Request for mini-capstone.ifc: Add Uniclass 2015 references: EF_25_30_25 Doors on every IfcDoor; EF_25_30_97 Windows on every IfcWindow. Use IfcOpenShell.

First a look at what the model holds.

```python
import ifcopenshell

model = ifcopenshell.open("mini-capstone.ifc")
print(model.schema)
print("classifications:", [c.Name for c in model.by_type("IfcClassification")])
for ifc_class in ("IfcDoor", "IfcRoof", "IfcStair", "IfcWall", "IfcWindow"):
    print(ifc_class, len(model.by_type(ifc_class)))
```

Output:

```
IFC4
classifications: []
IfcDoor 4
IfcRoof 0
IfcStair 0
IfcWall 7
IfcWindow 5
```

```python
import ifcopenshell
import ifcopenshell.api.classification

model = ifcopenshell.open("mini-capstone.ifc")

system = ifcopenshell.api.classification.add_classification(model, classification="Uniclass 2015")

codes = {
    "IfcDoor": ("EF_25_30_25", "Doors"),
    "IfcWindow": ("EF_25_30_97", "Windows"),
}
for ifc_class, (code, name) in codes.items():
    products = model.by_type(ifc_class)
    ifcopenshell.api.classification.add_reference(
        model, products=products, classification=system, identification=code, name=name
    )
    print(code, len(products))

model.write("mini-capstone_edited.ifc")
```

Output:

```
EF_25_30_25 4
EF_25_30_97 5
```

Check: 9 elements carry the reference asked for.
